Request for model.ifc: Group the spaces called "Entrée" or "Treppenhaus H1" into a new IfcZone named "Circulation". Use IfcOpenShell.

First a look at what the model holds.

```python
import ifcopenshell

model = ifcopenshell.open("model.ifc")
print(model.schema)
seen = {}
for space in model.by_type("IfcSpace"):
    seen[space.LongName] = seen.get(space.LongName, 0) + 1
for name, count in sorted(seen.items(), key=str):
    print(count, "x", name)
print("zones:", [z.Name for z in model.by_type("IfcZone")][:20])
```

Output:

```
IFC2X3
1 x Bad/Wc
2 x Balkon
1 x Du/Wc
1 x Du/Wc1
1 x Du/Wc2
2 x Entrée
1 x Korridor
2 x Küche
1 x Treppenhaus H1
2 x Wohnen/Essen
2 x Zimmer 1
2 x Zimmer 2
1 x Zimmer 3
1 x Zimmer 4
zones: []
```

```python
import ifcopenshell
import ifcopenshell.api.group
import ifcopenshell.api.root

model = ifcopenshell.open("model.ifc")

names = {"Entrée", "Treppenhaus H1"}
spaces = [s for s in model.by_type("IfcSpace") if s.LongName in names]

zone = ifcopenshell.api.root.create_entity(model, ifc_class="IfcZone", name="Circulation")
ifcopenshell.api.group.assign_group(model, products=spaces, group=zone)
print(len(spaces), "spaces in", zone.Name)

model.write("model_v2.ifc")
```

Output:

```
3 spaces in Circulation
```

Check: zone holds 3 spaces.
